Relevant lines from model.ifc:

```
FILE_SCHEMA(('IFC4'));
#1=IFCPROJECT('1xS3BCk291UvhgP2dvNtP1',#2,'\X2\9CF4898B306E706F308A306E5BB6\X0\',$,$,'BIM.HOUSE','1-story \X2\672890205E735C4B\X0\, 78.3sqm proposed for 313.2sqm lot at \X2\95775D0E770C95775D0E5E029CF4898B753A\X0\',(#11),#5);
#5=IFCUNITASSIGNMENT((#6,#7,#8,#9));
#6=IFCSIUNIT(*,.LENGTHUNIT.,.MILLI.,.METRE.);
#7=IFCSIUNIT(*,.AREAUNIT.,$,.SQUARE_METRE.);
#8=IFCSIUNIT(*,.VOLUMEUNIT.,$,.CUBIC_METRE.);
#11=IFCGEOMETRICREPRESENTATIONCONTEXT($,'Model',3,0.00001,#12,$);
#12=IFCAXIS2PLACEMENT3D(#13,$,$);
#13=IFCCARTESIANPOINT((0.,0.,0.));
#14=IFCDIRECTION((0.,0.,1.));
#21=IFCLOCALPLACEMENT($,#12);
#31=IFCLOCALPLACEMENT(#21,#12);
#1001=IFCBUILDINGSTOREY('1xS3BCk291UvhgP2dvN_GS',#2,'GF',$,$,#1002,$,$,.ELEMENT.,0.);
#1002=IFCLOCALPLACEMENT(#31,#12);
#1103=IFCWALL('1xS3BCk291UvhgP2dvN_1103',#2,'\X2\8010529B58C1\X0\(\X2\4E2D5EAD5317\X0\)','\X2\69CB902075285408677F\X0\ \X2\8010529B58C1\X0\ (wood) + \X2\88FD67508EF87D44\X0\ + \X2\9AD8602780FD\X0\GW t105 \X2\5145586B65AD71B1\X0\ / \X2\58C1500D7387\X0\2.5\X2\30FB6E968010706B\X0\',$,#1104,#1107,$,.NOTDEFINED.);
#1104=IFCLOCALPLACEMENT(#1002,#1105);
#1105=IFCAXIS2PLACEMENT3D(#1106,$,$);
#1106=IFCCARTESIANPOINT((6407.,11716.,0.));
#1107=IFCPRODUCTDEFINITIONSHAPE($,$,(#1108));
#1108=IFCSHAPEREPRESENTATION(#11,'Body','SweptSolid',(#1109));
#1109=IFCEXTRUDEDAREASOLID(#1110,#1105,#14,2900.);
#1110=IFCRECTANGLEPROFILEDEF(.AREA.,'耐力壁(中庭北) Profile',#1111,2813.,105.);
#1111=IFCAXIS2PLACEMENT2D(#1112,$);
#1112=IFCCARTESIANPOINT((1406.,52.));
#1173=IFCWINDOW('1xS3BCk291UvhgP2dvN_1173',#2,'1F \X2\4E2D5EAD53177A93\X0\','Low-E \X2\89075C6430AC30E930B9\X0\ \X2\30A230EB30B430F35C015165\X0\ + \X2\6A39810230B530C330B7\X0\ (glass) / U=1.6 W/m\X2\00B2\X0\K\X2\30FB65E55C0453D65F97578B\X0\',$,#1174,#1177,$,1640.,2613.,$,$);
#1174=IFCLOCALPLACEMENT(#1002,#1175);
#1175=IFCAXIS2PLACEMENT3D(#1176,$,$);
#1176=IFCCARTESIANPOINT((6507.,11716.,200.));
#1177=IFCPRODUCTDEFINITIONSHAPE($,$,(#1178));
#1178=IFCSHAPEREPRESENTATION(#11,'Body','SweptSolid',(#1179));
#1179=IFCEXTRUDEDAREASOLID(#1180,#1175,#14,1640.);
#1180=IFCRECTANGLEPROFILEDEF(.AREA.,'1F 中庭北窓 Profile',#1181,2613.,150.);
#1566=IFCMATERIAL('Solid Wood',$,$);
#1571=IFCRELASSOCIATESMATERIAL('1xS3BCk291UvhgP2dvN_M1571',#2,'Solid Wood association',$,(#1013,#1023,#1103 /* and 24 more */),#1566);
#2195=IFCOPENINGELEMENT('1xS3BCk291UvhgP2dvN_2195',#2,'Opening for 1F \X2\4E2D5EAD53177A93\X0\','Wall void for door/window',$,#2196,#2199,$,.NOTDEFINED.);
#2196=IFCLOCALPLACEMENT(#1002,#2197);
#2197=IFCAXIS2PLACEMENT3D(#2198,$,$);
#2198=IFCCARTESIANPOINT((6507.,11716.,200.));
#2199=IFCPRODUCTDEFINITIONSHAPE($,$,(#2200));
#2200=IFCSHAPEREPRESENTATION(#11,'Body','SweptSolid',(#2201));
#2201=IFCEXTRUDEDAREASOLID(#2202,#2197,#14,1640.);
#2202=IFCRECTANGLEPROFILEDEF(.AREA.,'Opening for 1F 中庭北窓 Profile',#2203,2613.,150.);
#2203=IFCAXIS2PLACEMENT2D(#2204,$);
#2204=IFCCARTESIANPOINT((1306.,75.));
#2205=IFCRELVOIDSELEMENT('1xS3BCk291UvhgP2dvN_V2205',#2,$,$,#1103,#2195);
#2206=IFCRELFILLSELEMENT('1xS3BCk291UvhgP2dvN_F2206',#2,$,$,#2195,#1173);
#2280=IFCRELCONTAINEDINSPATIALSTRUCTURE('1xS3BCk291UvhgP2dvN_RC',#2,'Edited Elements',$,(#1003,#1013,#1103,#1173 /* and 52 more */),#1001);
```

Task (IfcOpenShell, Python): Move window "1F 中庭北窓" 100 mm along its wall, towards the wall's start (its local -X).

```python
import ifcopenshell
import ifcopenshell.api.geometry
import ifcopenshell.util.placement

model = ifcopenshell.open("model.ifc")

window = model.by_guid("1xS3BCk291UvhgP2dvN_1173")
opening = window.FillsVoids[0].RelatingOpeningElement
wall = opening.VoidsElements[0].RelatingBuildingElement

wall_matrix = ifcopenshell.util.placement.get_local_placement(wall.ObjectPlacement)
shift = wall_matrix[:3, 0] * -100.0
before = ifcopenshell.util.placement.get_local_placement(window.ObjectPlacement)[:3, 3].copy()

# The window is not placed relative to its opening, so move both.
for product in (opening, window):
    matrix = ifcopenshell.util.placement.get_local_placement(product.ObjectPlacement)
    matrix[:3, 3] += shift
    ifcopenshell.api.geometry.edit_object_placement(model, product=product, matrix=matrix, is_si=False)

after = ifcopenshell.util.placement.get_local_placement(window.ObjectPlacement)[:3, 3]
print("window moved by", (after - before).round(3) + 0.0)

model.write("model_updated.ifc")
```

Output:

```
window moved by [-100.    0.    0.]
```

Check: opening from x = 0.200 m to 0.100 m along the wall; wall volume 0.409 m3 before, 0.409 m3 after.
